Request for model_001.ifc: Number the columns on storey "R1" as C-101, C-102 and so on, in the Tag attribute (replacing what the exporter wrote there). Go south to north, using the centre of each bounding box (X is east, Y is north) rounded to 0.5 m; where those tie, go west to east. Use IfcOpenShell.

First a look at what the model holds.

```python
import ifcopenshell
import ifcopenshell.util.element
import ifcopenshell.util.placement

model = ifcopenshell.open("model_001.ifc")
print(model.schema)
storey = next(s for s in model.by_type("IfcBuildingStorey") if s.Name == "R1")
columns = [e for e in ifcopenshell.util.element.get_decomposition(storey) if e.is_a("IfcColumn")]
for e in sorted(columns, key=lambda e: e.id()):
    origin = ifcopenshell.util.placement.get_local_placement(e.ObjectPlacement)[:3, 3]
    print(e.id(), e.Tag, e.Name, origin.round(2) + 0.0, sep=" | ")
```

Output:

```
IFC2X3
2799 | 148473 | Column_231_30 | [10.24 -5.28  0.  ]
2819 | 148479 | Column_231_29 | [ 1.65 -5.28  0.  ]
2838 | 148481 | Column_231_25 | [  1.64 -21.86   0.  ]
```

```python
import ifcopenshell
import ifcopenshell.geom
import ifcopenshell.util.element
import ifcopenshell.util.shape

model = ifcopenshell.open("model_001.ifc")
settings = ifcopenshell.geom.settings()
settings.set("use-world-coords", True)


def centre(element):
    shape = ifcopenshell.geom.create_shape(settings, element)
    return ifcopenshell.util.shape.get_bbox_centroid(shape.geometry)


storey = next(s for s in model.by_type("IfcBuildingStorey") if s.Name == "R1")
columns = [e for e in ifcopenshell.util.element.get_decomposition(storey) if e.is_a("IfcColumn")]

# Insertion points can sit at a corner or the storey origin, so sort by the geometry (in metres).
centres = {e: centre(e) for e in columns}
columns.sort(key=lambda e: (round(centres[e][1] / 0.5), centres[e][0]))

for i, e in enumerate(columns, start=1):
    number = f"C-1{i:02d}"
    e.Tag = number
    print(e.id(), number)

model.write("model_001_rev.ifc")
```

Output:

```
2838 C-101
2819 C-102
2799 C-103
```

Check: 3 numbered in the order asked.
